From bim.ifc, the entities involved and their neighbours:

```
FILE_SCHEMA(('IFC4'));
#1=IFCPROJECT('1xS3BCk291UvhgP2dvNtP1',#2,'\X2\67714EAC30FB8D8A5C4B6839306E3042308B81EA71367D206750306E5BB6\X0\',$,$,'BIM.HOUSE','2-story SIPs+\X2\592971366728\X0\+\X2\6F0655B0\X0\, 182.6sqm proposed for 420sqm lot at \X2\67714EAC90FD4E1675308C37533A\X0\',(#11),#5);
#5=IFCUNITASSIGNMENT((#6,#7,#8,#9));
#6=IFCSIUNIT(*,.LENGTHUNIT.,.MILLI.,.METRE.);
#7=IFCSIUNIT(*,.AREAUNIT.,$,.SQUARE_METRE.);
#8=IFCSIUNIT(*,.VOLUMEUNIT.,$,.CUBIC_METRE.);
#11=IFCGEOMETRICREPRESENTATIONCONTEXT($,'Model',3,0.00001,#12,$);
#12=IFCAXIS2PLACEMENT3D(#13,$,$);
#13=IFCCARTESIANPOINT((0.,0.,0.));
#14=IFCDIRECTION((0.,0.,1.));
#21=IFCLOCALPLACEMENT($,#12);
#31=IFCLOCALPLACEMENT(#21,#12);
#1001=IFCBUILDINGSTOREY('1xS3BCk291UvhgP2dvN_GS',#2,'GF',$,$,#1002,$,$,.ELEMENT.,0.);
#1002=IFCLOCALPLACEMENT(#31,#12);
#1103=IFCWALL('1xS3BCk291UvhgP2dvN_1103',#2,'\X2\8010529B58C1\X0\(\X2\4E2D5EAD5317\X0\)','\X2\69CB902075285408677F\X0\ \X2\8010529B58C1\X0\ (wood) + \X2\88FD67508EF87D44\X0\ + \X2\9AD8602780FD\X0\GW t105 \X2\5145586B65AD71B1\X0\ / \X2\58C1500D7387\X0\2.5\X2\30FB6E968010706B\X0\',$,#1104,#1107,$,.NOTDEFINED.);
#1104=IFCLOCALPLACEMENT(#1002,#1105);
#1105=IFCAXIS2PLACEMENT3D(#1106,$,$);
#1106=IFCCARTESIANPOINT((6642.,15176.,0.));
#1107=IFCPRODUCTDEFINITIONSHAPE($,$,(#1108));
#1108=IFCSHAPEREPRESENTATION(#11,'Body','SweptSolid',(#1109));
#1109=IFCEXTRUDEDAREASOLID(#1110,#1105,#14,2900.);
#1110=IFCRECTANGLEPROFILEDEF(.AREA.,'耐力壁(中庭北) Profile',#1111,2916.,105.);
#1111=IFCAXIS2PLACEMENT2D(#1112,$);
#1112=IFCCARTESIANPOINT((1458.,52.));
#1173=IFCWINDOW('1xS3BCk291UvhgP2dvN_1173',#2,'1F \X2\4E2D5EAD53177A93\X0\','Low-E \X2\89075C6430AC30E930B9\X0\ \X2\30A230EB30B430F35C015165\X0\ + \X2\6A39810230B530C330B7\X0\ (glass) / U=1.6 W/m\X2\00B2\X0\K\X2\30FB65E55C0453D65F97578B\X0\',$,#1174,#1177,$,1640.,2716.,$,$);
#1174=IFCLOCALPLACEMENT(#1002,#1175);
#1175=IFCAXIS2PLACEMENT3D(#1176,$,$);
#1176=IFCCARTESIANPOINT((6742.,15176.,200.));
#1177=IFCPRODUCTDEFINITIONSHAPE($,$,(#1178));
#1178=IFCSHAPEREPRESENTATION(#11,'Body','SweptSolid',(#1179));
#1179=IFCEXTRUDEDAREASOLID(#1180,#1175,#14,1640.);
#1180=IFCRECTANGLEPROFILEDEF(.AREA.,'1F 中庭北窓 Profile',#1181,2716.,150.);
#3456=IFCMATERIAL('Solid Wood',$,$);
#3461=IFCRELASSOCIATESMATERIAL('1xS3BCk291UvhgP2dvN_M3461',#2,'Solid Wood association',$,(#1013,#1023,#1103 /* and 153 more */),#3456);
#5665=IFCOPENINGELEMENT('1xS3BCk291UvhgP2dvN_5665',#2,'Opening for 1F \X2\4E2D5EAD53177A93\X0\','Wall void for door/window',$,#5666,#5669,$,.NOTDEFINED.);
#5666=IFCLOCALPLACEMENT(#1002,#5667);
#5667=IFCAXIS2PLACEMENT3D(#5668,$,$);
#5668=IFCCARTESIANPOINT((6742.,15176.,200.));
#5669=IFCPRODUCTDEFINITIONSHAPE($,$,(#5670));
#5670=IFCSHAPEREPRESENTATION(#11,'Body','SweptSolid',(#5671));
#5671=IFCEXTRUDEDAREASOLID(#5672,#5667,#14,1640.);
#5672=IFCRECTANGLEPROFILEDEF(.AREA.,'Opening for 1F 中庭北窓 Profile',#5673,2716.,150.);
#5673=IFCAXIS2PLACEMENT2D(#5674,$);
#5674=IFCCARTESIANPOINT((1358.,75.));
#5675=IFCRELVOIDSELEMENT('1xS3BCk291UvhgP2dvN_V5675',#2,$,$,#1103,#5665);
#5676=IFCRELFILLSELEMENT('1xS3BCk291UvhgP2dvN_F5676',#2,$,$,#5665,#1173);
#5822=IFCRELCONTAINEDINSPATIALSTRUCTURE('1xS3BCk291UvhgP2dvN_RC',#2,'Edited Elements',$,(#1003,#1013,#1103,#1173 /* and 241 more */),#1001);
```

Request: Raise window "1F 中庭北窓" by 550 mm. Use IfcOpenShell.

```python
import numpy as np
import ifcopenshell
import ifcopenshell.api.geometry
import ifcopenshell.util.placement
import ifcopenshell.util.unit

model = ifcopenshell.open("bim.ifc")
unit_scale = ifcopenshell.util.unit.calculate_unit_scale(model)

window = model.by_id(1173)
opening = window.FillsVoids[0].RelatingOpeningElement
dz = 550.0

shift = np.array([0.0, 0.0, dz])
# The window is not placed relative to its opening, so move both.
for product in (opening, window):
    matrix = ifcopenshell.util.placement.get_local_placement(product.ObjectPlacement)
    matrix[:3, 3] += shift
    ifcopenshell.api.geometry.edit_object_placement(model, product=product, matrix=matrix, is_si=False)

print(f"moved by {dz * unit_scale:+.3f} m")

model.write("bim_rev.ifc")
```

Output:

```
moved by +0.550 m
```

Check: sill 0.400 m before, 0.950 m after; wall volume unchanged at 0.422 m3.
